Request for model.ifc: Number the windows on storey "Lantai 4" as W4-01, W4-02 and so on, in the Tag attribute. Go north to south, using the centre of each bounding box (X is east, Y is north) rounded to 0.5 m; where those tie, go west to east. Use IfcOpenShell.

First a look at what the model holds.

```python
import ifcopenshell
import ifcopenshell.util.element
import ifcopenshell.util.placement

model = ifcopenshell.open("model.ifc")
print(model.schema)
storey = next(s for s in model.by_type("IfcBuildingStorey") if s.Name == "Lantai 4")
windows = [e for e in ifcopenshell.util.element.get_decomposition(storey) if e.is_a("IfcWindow")]
for e in sorted(windows, key=lambda e: e.id()):
    origin = ifcopenshell.util.placement.get_local_placement(e.ObjectPlacement)[:3, 3]
    print(e.id(), e.Tag, e.Name, origin.round(2) + 0.0, sep=" | ")
```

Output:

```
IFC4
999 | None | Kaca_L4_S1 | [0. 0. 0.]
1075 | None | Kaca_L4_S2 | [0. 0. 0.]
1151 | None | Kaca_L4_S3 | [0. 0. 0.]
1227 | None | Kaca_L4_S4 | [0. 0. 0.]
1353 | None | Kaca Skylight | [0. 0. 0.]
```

```python
import ifcopenshell
import ifcopenshell.geom
import ifcopenshell.util.element
import ifcopenshell.util.shape

model = ifcopenshell.open("model.ifc")
settings = ifcopenshell.geom.settings()
settings.set("use-world-coords", True)


def centre(element):
    shape = ifcopenshell.geom.create_shape(settings, element)
    return ifcopenshell.util.shape.get_bbox_centroid(shape.geometry)


storey = next(s for s in model.by_type("IfcBuildingStorey") if s.Name == "Lantai 4")
windows = [e for e in ifcopenshell.util.element.get_decomposition(storey) if e.is_a("IfcWindow")]

# Insertion points can sit at a corner or the storey origin, so sort by the geometry (in metres).
centres = {e: centre(e) for e in windows}
windows.sort(key=lambda e: (-round(centres[e][1] / 0.5), centres[e][0]))

for i, e in enumerate(windows, start=1):
    number = f"W4-{i:02d}"
    e.Tag = number
    print(e.id(), number)

model.write("model_v2.ifc")
```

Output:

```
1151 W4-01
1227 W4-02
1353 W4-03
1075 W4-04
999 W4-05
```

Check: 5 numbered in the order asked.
